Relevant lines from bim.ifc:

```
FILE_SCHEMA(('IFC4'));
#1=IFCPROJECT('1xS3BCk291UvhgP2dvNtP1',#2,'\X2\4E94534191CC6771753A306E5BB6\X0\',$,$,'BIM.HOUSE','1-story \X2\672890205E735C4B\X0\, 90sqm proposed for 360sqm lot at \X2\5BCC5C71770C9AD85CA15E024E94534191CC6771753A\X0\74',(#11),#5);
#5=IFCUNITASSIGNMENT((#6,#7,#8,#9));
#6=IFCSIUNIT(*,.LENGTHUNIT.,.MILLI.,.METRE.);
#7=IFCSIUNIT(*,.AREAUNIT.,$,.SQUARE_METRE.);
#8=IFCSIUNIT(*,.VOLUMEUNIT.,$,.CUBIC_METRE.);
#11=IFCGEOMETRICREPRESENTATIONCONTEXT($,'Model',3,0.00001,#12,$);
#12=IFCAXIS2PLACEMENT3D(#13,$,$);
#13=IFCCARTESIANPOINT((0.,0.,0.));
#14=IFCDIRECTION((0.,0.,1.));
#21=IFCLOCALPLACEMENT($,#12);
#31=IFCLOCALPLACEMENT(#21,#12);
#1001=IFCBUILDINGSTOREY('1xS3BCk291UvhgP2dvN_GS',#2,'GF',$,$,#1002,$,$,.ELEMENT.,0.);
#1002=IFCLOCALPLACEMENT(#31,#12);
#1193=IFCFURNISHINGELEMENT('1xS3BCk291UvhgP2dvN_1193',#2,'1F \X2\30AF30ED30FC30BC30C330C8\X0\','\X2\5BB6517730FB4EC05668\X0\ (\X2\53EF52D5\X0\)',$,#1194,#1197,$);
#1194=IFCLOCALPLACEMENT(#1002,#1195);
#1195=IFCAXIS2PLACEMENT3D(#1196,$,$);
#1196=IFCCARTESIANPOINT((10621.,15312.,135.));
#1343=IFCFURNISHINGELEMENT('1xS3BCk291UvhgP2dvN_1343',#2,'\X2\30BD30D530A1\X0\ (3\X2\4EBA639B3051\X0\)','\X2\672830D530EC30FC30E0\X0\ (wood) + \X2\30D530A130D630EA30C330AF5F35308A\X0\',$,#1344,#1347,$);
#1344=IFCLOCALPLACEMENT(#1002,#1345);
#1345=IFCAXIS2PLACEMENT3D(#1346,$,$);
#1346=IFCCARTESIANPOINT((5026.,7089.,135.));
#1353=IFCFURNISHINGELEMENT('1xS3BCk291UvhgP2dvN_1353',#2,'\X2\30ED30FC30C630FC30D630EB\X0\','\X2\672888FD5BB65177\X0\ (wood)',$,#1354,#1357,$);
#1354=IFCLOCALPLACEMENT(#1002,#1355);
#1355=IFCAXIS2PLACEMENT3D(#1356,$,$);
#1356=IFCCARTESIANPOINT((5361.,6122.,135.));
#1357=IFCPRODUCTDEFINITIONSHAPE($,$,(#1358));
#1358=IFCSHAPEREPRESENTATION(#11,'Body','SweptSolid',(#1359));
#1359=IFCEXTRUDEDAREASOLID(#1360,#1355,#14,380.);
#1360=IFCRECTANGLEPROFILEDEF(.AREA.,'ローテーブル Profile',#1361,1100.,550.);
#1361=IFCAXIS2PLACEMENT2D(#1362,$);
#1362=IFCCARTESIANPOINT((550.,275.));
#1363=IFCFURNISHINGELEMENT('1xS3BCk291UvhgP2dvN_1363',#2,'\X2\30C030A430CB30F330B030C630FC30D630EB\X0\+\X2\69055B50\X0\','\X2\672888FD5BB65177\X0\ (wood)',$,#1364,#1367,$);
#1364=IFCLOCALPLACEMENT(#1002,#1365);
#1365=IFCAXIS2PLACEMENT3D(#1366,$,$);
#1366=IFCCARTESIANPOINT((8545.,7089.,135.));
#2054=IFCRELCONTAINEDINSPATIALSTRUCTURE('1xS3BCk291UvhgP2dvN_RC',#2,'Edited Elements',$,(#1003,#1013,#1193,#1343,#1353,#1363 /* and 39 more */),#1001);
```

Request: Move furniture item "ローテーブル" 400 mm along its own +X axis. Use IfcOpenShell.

```python
import ifcopenshell
import ifcopenshell.api.geometry
import ifcopenshell.util.placement

model = ifcopenshell.open("bim.ifc")

item = model.by_guid("1xS3BCk291UvhgP2dvN_1353")
matrix = ifcopenshell.util.placement.get_local_placement(item.ObjectPlacement)
matrix[:3, 3] += matrix[:3, 0] * 400.0
ifcopenshell.api.geometry.edit_object_placement(model, product=item, matrix=matrix, is_si=False)

print(ifcopenshell.util.placement.get_local_placement(item.ObjectPlacement).round(3) + 0.0)

model.write("bim_v2.ifc")
```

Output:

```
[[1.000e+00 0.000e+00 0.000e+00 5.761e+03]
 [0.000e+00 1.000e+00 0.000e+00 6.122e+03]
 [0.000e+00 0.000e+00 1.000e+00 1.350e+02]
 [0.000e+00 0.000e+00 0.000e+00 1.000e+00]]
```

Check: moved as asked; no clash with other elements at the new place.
